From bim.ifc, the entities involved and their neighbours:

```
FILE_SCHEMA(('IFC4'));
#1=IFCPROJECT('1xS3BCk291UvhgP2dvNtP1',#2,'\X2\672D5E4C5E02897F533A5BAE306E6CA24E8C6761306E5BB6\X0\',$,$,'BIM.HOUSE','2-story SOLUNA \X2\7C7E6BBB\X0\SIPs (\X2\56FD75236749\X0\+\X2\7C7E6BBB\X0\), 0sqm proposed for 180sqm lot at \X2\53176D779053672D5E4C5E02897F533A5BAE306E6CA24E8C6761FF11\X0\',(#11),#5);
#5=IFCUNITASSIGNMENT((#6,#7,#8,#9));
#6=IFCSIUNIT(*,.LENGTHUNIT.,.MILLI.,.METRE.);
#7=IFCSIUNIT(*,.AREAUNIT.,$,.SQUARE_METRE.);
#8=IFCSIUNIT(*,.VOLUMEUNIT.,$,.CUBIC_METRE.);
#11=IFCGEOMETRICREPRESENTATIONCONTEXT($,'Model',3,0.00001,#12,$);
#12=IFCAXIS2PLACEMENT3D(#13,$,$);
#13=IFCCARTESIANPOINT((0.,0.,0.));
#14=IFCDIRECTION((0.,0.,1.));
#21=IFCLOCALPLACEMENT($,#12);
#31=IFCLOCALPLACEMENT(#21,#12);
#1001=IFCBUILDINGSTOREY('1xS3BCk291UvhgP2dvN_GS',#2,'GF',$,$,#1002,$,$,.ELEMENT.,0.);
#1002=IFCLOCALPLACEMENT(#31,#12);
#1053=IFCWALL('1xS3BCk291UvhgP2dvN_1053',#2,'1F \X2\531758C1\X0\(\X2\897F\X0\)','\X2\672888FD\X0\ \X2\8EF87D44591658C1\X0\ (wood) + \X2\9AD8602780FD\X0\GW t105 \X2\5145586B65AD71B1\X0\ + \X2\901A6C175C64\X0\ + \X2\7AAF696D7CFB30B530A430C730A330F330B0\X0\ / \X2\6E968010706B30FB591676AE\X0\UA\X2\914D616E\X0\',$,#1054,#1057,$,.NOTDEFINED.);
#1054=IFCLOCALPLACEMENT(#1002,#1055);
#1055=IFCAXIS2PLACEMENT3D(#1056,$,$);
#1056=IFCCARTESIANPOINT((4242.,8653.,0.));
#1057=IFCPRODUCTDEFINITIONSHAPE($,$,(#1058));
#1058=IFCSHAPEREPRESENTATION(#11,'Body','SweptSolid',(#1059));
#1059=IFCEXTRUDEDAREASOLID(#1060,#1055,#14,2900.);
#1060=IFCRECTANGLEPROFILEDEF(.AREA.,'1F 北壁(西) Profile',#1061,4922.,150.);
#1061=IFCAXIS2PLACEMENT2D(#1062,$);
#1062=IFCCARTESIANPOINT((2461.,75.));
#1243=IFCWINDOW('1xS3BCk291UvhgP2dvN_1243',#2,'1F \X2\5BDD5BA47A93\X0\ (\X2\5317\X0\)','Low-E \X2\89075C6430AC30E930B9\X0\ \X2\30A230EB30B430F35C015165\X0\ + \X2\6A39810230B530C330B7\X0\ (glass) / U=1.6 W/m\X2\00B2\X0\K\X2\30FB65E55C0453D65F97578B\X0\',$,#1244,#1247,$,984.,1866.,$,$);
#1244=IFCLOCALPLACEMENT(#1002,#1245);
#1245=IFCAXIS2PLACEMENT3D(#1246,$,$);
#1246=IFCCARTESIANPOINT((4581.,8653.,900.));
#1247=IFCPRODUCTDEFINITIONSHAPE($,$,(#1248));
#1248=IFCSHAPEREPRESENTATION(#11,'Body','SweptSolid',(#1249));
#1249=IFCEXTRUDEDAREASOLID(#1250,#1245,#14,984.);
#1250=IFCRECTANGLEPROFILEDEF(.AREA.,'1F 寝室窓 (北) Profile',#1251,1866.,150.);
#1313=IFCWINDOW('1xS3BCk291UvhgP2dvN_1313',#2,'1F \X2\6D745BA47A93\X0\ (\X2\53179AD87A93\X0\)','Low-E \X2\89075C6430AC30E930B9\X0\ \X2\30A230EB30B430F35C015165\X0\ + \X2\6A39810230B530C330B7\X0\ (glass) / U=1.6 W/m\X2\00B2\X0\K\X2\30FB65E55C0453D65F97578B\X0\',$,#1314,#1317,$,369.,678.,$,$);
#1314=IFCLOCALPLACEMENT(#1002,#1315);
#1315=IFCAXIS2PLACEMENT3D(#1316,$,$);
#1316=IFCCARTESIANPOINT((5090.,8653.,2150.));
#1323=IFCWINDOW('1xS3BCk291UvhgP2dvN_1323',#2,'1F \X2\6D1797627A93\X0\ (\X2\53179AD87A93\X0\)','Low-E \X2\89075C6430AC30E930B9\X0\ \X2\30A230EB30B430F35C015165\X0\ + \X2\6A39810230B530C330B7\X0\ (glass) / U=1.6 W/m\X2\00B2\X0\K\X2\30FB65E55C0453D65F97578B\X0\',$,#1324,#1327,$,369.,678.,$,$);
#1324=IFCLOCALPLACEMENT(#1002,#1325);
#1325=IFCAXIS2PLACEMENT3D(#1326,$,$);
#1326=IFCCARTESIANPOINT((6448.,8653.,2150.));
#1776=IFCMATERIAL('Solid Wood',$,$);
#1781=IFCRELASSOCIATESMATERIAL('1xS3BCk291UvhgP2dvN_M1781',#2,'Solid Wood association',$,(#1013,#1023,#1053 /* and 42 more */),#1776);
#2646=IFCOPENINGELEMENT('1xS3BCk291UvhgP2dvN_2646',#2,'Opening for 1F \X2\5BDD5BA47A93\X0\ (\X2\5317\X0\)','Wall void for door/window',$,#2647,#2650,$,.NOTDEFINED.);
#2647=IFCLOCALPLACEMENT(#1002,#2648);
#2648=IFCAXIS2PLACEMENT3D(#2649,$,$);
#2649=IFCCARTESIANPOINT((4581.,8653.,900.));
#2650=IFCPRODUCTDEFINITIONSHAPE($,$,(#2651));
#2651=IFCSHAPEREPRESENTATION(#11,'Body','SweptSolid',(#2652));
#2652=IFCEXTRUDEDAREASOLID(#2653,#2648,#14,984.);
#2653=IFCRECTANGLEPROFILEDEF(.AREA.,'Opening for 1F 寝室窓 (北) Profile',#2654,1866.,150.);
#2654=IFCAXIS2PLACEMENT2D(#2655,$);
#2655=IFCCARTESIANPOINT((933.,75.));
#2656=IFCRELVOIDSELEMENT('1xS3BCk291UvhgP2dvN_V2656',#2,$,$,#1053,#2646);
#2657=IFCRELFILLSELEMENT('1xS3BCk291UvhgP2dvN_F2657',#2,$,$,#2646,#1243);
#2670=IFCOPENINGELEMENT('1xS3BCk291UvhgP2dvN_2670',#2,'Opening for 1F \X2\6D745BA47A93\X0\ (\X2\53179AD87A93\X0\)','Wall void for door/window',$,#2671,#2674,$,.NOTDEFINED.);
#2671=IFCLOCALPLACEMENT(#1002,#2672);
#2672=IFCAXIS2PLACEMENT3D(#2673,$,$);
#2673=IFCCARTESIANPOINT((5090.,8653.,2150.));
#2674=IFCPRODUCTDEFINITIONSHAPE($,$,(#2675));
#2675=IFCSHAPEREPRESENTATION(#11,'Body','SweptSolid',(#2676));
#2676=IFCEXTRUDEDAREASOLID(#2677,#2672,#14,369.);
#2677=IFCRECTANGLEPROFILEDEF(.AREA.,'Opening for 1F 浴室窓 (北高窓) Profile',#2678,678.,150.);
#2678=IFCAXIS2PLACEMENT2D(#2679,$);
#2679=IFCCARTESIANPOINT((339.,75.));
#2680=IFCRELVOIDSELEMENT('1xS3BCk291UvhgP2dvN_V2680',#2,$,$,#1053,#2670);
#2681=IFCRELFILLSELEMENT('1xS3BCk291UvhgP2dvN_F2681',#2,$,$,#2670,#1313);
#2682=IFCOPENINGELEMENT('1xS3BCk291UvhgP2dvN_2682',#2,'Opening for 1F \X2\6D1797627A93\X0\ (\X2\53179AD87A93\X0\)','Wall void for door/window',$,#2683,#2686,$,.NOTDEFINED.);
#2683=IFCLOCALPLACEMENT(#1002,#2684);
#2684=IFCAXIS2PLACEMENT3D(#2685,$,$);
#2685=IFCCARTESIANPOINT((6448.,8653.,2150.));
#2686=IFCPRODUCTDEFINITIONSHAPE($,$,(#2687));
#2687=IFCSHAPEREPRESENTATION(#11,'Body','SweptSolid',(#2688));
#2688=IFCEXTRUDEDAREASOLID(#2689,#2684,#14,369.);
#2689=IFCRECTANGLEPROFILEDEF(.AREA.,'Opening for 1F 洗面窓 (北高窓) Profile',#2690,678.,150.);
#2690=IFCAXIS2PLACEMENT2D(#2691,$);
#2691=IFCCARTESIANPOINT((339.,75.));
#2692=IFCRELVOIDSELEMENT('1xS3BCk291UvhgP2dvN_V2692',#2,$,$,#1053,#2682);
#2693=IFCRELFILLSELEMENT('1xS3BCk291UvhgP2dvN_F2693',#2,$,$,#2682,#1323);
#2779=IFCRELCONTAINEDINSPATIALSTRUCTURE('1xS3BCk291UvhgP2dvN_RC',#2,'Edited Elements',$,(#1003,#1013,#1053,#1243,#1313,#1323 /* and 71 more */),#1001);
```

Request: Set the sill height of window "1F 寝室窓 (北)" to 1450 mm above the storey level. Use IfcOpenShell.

```python
import numpy as np
import ifcopenshell
import ifcopenshell.api.geometry
import ifcopenshell.geom
import ifcopenshell.util.element
import ifcopenshell.util.placement
import ifcopenshell.util.shape
import ifcopenshell.util.unit

model = ifcopenshell.open("bim.ifc")
unit_scale = ifcopenshell.util.unit.calculate_unit_scale(model)

window = model.by_guid("1xS3BCk291UvhgP2dvN_1243")
opening = window.FillsVoids[0].RelatingOpeningElement
storey = ifcopenshell.util.element.get_container(window, ifc_class="IfcBuildingStorey")
level = ifcopenshell.util.placement.get_local_placement(storey.ObjectPlacement)[2, 3]

# The opening's origin need not be at the sill, so measure its lowest point.
shape = ifcopenshell.geom.create_shape(ifcopenshell.geom.settings(), opening)
bottom = ifcopenshell.util.shape.get_shape_bottom_elevation(shape, shape.geometry) / unit_scale
dz = level + 1.45 / unit_scale - bottom

shift = np.array([0.0, 0.0, dz])
# The window is not placed relative to its opening, so move both.
for product in (opening, window):
    matrix = ifcopenshell.util.placement.get_local_placement(product.ObjectPlacement)
    matrix[:3, 3] += shift
    ifcopenshell.api.geometry.edit_object_placement(model, product=product, matrix=matrix, is_si=False)

print(f"moved by {dz * unit_scale:+.3f} m")

model.write("bim-out.ifc")
```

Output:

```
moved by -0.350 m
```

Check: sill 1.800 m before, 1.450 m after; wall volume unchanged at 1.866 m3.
